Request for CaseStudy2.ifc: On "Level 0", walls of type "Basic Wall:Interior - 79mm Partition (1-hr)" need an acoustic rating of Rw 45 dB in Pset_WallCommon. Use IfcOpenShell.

First a look at what the model holds.

```python
import ifcopenshell
import ifcopenshell.util.element

model = ifcopenshell.open("CaseStudy2.ifc")
print(model.schema)
storey = next(s for s in model.by_type("IfcBuildingStorey") if s.Name == "Level 0")
walls = [e for e in ifcopenshell.util.element.get_decomposition(storey) if e.is_a("IfcWall")]
seen = {}
for e in walls:
    element_type = ifcopenshell.util.element.get_type(e)
    key = (element_type.Name if element_type != e and element_type else None, ifcopenshell.util.element.get_pset(e, "Pset_WallCommon", "AcousticRating"))
    seen[key] = seen.get(key, 0) + 1
for (name, value), count in sorted(seen.items(), key=str):
    print(count, "x", name, "|", value)
```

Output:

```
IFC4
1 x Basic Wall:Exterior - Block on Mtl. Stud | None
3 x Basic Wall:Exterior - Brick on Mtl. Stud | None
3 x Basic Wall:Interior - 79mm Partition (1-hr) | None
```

```python
import ifcopenshell
import ifcopenshell.api.pset
import ifcopenshell.util.element

model = ifcopenshell.open("CaseStudy2.ifc")

storey = next(s for s in model.by_type("IfcBuildingStorey") if s.Name == "Level 0")
walls = [e for e in ifcopenshell.util.element.get_decomposition(storey) if e.is_a("IfcWall")]

count = 0
for e in walls:
    element_type = ifcopenshell.util.element.get_type(e)
    if element_type in (None, e) or element_type.Name != "Basic Wall:Interior - 79mm Partition (1-hr)":
        continue
    # add_pset returns the element's existing set when there is one.
    pset = ifcopenshell.api.pset.add_pset(model, product=e, name="Pset_WallCommon")
    ifcopenshell.api.pset.edit_pset(model, pset=pset, properties={"AcousticRating": "Rw 45 dB"})
    count += 1

print(count, "walls updated")

model.write("CaseStudy2_edited.ifc")
```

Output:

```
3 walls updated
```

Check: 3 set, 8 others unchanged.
